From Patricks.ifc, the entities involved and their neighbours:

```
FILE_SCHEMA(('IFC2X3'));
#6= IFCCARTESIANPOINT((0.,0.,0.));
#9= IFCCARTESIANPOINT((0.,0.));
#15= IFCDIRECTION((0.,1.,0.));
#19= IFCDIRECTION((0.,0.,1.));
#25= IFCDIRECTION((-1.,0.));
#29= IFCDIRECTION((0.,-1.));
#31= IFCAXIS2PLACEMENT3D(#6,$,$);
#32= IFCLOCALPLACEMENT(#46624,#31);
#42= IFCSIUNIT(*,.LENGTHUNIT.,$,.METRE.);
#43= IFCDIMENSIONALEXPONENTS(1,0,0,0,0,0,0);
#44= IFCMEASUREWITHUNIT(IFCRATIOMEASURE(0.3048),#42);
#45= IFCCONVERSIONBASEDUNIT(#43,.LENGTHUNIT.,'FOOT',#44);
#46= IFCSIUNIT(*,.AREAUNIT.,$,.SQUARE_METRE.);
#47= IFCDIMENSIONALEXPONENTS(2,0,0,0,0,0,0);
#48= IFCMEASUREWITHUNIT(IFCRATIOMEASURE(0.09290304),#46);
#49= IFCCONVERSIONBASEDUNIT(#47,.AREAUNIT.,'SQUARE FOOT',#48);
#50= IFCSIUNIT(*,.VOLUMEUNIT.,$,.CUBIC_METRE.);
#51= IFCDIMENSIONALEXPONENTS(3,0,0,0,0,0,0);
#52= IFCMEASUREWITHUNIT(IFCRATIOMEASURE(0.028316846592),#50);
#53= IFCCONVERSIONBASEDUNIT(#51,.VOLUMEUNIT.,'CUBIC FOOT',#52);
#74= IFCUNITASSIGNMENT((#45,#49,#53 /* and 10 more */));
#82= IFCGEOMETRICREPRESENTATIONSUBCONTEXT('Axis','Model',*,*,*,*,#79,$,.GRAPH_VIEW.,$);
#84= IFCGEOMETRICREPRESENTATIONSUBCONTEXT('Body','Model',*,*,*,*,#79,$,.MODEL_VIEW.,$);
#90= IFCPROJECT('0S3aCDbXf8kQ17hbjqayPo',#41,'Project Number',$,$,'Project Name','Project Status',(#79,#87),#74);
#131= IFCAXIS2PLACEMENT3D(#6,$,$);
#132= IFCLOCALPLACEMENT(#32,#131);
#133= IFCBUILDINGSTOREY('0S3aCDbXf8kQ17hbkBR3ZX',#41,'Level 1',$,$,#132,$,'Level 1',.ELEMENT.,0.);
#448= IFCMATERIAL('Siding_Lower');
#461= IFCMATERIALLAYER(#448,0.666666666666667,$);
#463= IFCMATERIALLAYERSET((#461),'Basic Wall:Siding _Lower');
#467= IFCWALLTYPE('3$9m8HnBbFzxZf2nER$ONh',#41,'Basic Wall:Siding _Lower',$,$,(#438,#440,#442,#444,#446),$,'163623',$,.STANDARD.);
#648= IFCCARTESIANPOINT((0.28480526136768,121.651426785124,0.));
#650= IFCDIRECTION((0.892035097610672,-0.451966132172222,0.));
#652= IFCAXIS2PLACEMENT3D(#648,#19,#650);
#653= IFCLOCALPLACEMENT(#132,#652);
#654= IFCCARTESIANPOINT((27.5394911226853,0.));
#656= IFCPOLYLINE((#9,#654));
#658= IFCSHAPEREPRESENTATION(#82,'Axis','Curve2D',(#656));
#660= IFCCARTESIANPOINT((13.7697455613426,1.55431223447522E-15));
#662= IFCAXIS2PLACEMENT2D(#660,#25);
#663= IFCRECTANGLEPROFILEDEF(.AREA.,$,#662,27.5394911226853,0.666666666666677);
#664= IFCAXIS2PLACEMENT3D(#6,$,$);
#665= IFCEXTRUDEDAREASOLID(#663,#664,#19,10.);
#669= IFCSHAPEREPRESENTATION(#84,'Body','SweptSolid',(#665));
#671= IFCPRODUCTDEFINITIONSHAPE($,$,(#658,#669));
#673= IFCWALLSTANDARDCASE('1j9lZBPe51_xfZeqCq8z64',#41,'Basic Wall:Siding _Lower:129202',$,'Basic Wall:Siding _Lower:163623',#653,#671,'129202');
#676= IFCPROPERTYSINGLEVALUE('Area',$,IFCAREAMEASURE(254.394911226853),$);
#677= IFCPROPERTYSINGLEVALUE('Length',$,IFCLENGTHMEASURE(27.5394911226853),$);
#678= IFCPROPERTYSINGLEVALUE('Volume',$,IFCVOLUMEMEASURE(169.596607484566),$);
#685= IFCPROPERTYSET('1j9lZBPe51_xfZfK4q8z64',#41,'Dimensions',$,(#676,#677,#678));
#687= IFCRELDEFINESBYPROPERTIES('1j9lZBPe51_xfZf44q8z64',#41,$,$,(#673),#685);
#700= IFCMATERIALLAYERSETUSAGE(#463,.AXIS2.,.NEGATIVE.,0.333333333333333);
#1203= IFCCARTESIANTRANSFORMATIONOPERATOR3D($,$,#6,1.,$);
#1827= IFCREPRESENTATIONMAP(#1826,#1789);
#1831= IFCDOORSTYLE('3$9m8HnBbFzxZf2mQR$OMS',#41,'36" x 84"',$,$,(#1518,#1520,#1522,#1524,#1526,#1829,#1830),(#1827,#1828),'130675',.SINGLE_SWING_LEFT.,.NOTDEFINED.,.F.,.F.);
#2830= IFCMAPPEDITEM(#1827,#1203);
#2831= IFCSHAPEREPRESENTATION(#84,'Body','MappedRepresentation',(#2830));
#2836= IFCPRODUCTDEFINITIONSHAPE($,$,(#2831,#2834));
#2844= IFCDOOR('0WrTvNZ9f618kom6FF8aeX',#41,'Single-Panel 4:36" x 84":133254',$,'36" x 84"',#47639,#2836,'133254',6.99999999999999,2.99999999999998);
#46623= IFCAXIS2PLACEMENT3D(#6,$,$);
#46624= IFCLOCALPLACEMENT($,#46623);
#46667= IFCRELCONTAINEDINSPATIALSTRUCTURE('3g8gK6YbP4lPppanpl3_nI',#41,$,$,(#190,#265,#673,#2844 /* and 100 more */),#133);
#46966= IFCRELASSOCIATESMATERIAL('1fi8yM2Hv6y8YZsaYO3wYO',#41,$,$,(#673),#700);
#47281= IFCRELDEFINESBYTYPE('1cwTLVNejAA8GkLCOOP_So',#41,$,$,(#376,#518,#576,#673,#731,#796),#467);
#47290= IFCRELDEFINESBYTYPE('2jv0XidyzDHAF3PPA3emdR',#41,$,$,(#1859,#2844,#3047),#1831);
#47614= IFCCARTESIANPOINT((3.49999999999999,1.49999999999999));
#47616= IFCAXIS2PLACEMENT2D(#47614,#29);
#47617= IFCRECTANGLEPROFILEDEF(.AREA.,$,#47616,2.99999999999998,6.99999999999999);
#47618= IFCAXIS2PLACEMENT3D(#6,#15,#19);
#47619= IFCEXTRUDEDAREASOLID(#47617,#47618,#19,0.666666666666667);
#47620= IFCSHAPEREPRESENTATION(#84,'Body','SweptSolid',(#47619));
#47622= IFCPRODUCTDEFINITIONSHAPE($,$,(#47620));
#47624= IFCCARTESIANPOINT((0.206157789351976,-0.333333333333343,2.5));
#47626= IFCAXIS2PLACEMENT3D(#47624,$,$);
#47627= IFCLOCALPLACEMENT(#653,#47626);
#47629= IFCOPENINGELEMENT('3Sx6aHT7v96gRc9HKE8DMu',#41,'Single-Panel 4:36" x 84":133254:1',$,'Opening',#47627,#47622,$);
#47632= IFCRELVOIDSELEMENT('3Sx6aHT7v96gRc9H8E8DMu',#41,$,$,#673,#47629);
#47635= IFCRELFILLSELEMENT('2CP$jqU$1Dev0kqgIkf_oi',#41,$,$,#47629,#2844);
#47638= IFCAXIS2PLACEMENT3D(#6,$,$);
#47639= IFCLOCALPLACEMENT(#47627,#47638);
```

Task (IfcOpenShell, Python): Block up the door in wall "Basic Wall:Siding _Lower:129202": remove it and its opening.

```python
import ifcopenshell
import ifcopenshell.api.feature
import ifcopenshell.api.pset
import ifcopenshell.api.root
import ifcopenshell.geom
import ifcopenshell.util.element
import ifcopenshell.util.shape
import ifcopenshell.util.unit

model = ifcopenshell.open("Patricks.ifc")
area_scale = ifcopenshell.util.unit.calculate_unit_scale(model, "AREAUNIT")
volume_scale = ifcopenshell.util.unit.calculate_unit_scale(model, "VOLUMEUNIT")
settings = ifcopenshell.geom.settings()


def volume(element):
    """Net volume in cubic metres, openings subtracted."""
    shape = ifcopenshell.geom.create_shape(settings, element)
    return ifcopenshell.util.shape.get_volume(shape.geometry)


door = model.by_guid("0WrTvNZ9f618kom6FF8aeX")
opening = door.FillsVoids[0].RelatingOpeningElement
wall = opening.VoidsElements[0].RelatingBuildingElement
before = volume(wall)

ifcopenshell.api.root.remove_product(model, product=door)
ifcopenshell.api.feature.remove_feature(model, feature=opening)

after = volume(wall)
thickness = 0.2032  # wall thickness in metres

# Update the wall's stored quantities.
pset = model.by_id(ifcopenshell.util.element.get_pset(wall, "Dimensions", should_inherit=False)["id"])
ifcopenshell.api.pset.edit_pset(model, pset=pset, properties={
    "Area": model.create_entity("IfcAreaMeasure", after / thickness / area_scale),
    "Volume": model.create_entity("IfcVolumeMeasure", after / volume_scale),
})

print(f"wall volume {before:.3f} -> {after:.3f} m3")

model.write("Patricks-out.ifc")
```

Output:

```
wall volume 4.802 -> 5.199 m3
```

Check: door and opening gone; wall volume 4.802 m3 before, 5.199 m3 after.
